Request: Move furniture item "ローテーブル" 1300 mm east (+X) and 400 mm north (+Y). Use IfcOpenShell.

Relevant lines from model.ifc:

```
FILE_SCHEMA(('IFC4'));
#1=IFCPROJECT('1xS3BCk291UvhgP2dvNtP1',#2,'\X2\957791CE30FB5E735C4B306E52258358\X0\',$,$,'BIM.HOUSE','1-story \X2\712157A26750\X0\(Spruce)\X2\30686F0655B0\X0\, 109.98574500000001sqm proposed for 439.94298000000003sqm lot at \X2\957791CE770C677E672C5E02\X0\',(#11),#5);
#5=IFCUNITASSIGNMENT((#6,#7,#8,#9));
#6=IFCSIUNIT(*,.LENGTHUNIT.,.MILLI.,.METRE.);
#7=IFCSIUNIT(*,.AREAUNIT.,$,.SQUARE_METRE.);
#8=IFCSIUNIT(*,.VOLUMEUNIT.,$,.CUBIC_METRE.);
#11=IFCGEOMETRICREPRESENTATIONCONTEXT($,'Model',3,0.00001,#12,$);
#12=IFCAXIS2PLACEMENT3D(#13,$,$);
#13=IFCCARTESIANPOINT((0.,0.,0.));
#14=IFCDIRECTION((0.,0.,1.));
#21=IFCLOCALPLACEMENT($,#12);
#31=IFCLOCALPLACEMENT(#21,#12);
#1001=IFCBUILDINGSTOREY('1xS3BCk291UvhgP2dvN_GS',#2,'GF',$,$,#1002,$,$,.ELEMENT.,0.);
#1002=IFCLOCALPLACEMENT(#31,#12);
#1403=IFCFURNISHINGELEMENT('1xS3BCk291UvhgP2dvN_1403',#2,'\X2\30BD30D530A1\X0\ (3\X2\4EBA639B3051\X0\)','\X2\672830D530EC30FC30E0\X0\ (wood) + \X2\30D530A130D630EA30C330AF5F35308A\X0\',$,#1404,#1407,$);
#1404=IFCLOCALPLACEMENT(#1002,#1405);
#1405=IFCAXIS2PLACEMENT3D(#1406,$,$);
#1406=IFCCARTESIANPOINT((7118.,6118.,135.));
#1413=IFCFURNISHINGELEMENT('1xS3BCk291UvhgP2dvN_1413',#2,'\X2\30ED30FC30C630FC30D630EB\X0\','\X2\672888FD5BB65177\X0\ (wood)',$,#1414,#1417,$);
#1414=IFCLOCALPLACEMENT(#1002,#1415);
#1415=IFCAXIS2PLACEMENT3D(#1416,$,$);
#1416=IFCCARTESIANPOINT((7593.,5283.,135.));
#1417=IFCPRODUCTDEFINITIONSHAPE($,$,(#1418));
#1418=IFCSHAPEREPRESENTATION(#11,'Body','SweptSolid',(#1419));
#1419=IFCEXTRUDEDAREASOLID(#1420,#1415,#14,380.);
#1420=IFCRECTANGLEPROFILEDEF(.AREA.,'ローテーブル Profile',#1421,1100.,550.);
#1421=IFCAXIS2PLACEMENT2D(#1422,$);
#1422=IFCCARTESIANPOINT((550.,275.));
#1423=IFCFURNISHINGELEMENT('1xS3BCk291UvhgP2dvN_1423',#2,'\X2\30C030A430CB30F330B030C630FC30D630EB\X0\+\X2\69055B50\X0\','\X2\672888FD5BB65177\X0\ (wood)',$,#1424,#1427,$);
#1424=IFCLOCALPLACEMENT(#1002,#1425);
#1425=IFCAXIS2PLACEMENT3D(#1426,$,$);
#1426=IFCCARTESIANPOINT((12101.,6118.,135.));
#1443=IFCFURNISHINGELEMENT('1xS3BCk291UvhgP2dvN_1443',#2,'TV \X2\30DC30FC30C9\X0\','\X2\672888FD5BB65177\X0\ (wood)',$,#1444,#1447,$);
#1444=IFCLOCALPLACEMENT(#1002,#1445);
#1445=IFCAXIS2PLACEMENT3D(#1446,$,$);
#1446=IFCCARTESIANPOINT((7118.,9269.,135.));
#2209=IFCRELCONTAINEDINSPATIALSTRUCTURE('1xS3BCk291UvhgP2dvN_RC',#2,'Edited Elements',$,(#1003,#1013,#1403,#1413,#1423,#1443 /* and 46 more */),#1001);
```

```python
import ifcopenshell
import ifcopenshell.api.geometry
import ifcopenshell.util.placement

model = ifcopenshell.open("model.ifc")

item = model.by_id(1413)
matrix = ifcopenshell.util.placement.get_local_placement(item.ObjectPlacement)
matrix[0, 3] += 1300.0
matrix[1, 3] += 400.0
ifcopenshell.api.geometry.edit_object_placement(model, product=item, matrix=matrix, is_si=False)

print(ifcopenshell.util.placement.get_local_placement(item.ObjectPlacement).round(3) + 0.0)

model.write("model-out.ifc")
```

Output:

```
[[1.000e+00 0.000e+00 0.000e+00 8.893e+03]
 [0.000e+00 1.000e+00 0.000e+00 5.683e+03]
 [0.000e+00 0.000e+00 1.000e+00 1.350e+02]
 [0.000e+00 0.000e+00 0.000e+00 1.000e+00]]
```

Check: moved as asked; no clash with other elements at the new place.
